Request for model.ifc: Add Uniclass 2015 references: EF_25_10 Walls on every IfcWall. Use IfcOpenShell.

First a look at what the model holds.

```python
import ifcopenshell

model = ifcopenshell.open("model.ifc")
print(model.schema)
print("classifications:", [c.Name for c in model.by_type("IfcClassification")])
for ifc_class in ("IfcDoor", "IfcRoof", "IfcStair", "IfcWall", "IfcWindow"):
    print(ifc_class, len(model.by_type(ifc_class)))
```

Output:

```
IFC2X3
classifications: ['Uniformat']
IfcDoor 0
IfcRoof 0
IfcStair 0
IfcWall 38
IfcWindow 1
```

```python
import ifcopenshell
import ifcopenshell.api.classification

model = ifcopenshell.open("model.ifc")

# IFC2X3 requires Source and Edition and has no link from the project to the system.
system = model.create_entity("IfcClassification", Source="NBS", Edition="2015", Name="Uniclass 2015")

codes = {
    "IfcWall": ("EF_25_10", "Walls"),
}
for ifc_class, (code, name) in codes.items():
    products = model.by_type(ifc_class)
    ifcopenshell.api.classification.add_reference(
        model, products=products, classification=system, identification=code, name=name
    )
    print(code, len(products))

model.write("model_v2.ifc")
```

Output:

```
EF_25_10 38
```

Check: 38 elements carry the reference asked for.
